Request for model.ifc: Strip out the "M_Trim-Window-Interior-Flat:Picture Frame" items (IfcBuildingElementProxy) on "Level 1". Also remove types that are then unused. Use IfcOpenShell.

First a look at what the model holds.

```python
import ifcopenshell
import ifcopenshell.util.element

model = ifcopenshell.open("model.ifc")
print(model.schema)
storey = next(s for s in model.by_type("IfcBuildingStorey") if s.Name == "Level 1")
proxies = [e for e in ifcopenshell.util.element.get_decomposition(storey) if e.is_a("IfcBuildingElementProxy")]
seen = {}
for e in proxies:
    element_type = ifcopenshell.util.element.get_type(e)
    name = element_type.Name if element_type not in (None, e) else None
    seen[name] = seen.get(name, 0) + 1
for name, count in sorted(seen.items(), key=str):
    print(count, "x", name)
```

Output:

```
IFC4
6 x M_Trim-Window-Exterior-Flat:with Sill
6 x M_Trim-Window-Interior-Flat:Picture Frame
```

```python
import ifcopenshell
import ifcopenshell.api.root
import ifcopenshell.util.element

model = ifcopenshell.open("model.ifc")

storey = next(s for s in model.by_type("IfcBuildingStorey") if s.Name == "Level 1")
proxies = [e for e in ifcopenshell.util.element.get_decomposition(storey) if e.is_a("IfcBuildingElementProxy")]
targets = [e for e in proxies if (t := ifcopenshell.util.element.get_type(e)) not in (None, e) and t.Name == "M_Trim-Window-Interior-Flat:Picture Frame"]
types = {ifcopenshell.util.element.get_type(e) for e in targets} - {None, *targets}

for e in targets:
    ifcopenshell.api.root.remove_product(model, product=e)
print(len(targets), "removed")

unused = [t for t in types if not ifcopenshell.util.element.get_types(t)]
for t in unused:
    ifcopenshell.api.root.remove_product(model, product=t)
print(len(unused), "unused types removed")

model.write("model_updated.ifc")
```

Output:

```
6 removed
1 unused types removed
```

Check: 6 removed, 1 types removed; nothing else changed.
